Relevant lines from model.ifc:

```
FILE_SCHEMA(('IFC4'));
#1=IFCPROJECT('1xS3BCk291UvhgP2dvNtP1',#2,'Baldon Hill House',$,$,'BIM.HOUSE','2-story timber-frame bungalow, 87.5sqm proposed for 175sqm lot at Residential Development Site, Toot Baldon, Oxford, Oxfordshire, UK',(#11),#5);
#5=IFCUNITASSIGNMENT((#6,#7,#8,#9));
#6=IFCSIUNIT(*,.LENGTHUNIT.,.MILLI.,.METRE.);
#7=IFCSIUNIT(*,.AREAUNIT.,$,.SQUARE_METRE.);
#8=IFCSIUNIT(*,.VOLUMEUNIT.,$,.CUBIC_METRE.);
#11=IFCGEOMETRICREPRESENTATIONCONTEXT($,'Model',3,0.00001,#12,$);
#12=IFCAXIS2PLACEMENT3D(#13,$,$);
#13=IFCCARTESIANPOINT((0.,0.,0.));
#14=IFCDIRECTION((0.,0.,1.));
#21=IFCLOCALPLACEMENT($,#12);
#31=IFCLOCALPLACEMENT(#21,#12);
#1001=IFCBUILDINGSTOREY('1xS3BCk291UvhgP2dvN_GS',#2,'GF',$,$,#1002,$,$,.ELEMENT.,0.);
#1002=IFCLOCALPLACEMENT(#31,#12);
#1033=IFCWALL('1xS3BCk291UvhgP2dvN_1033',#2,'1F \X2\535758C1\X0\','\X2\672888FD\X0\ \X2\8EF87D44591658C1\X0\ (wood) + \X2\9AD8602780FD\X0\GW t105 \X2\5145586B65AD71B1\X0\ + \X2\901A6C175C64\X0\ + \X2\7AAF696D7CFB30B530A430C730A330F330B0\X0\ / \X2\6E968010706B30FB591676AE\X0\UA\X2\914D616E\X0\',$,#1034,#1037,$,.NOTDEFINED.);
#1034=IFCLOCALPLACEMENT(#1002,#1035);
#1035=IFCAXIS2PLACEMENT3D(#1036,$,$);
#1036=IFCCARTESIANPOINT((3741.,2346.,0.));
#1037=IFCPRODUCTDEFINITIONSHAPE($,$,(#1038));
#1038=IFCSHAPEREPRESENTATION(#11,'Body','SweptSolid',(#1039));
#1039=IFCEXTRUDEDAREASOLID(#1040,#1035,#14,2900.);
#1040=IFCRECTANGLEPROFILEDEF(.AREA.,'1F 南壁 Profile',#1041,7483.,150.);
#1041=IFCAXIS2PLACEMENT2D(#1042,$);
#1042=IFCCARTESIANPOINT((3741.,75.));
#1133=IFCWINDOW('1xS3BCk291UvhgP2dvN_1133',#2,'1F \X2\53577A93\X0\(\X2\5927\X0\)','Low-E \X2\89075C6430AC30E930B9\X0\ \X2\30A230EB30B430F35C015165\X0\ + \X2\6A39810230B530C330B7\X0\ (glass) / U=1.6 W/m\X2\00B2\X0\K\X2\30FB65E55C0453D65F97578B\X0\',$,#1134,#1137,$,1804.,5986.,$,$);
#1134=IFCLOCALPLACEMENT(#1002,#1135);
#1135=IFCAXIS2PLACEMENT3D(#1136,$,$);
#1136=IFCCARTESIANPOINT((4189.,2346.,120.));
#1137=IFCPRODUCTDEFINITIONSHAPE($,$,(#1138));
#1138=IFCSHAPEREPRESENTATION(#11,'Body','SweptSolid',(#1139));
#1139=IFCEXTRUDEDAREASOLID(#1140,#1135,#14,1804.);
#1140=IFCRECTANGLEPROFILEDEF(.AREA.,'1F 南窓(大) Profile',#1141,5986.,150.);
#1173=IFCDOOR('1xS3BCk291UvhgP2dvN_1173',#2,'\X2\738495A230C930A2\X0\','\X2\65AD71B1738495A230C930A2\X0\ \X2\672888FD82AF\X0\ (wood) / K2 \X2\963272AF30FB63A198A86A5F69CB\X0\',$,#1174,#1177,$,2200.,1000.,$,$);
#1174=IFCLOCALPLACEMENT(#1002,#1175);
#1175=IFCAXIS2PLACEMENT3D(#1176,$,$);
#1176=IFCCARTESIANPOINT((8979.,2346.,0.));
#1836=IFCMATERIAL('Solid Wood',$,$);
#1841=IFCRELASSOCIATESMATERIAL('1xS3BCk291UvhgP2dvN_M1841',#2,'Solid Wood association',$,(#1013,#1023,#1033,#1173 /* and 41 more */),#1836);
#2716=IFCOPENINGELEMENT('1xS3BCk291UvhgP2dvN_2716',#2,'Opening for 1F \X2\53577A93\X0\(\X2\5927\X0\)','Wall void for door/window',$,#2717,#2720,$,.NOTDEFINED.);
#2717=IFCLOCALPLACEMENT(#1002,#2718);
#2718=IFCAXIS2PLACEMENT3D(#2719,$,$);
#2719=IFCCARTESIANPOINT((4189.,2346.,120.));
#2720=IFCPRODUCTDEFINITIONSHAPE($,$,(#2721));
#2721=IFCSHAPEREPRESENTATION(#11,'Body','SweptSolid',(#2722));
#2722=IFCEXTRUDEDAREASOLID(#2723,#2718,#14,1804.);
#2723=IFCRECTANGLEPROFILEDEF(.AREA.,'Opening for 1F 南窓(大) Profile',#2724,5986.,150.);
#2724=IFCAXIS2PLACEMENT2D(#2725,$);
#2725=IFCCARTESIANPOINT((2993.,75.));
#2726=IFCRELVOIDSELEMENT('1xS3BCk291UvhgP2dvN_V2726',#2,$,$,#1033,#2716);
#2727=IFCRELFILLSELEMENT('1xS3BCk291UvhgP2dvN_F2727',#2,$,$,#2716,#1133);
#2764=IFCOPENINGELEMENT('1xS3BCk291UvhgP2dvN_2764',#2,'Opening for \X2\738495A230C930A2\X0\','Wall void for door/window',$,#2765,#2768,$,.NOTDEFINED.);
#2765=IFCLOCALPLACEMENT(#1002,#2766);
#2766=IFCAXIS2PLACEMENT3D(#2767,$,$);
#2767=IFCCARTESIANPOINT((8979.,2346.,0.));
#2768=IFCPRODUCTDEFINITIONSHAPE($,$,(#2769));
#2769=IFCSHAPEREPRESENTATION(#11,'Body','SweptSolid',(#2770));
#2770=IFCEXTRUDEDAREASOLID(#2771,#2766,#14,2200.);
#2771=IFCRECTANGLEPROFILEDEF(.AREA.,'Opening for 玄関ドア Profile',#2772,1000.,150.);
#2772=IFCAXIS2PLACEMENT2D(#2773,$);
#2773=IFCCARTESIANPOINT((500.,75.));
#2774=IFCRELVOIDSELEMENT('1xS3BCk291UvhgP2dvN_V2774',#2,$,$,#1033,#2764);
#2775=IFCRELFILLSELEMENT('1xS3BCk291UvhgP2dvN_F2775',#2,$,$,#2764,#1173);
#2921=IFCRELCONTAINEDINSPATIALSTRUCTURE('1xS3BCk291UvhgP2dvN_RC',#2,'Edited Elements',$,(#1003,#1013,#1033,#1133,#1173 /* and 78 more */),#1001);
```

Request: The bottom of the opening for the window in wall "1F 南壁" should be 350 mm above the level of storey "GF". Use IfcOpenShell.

```python
import numpy as np
import ifcopenshell
import ifcopenshell.api.geometry
import ifcopenshell.geom
import ifcopenshell.util.element
import ifcopenshell.util.placement
import ifcopenshell.util.shape
import ifcopenshell.util.unit

model = ifcopenshell.open("model.ifc")
unit_scale = ifcopenshell.util.unit.calculate_unit_scale(model)

window = model.by_guid("1xS3BCk291UvhgP2dvN_1133")
opening = window.FillsVoids[0].RelatingOpeningElement
storey = ifcopenshell.util.element.get_container(window, ifc_class="IfcBuildingStorey")
level = ifcopenshell.util.placement.get_local_placement(storey.ObjectPlacement)[2, 3]

# The opening's origin need not be at the sill, so measure its lowest point.
shape = ifcopenshell.geom.create_shape(ifcopenshell.geom.settings(), opening)
bottom = ifcopenshell.util.shape.get_shape_bottom_elevation(shape, shape.geometry) / unit_scale
dz = level + 0.35 / unit_scale - bottom

shift = np.array([0.0, 0.0, dz])
# The window is not placed relative to its opening, so move both.
for product in (opening, window):
    matrix = ifcopenshell.util.placement.get_local_placement(product.ObjectPlacement)
    matrix[:3, 3] += shift
    ifcopenshell.api.geometry.edit_object_placement(model, product=product, matrix=matrix, is_si=False)

print(f"moved by {dz * unit_scale:+.3f} m")

model.write("model_rev.ifc")
```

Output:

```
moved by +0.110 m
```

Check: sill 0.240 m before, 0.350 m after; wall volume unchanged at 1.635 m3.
